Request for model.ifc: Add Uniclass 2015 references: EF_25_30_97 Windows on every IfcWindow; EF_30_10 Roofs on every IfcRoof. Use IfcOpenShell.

First a look at what the model holds.

```python
import ifcopenshell

model = ifcopenshell.open("model.ifc")
print(model.schema)
print("classifications:", [c.Name for c in model.by_type("IfcClassification")])
for ifc_class in ("IfcDoor", "IfcRoof", "IfcStair", "IfcWall", "IfcWindow"):
    print(ifc_class, len(model.by_type(ifc_class)))
```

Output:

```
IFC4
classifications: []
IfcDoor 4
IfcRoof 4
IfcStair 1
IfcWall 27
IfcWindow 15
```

```python
import ifcopenshell
import ifcopenshell.api.classification

model = ifcopenshell.open("model.ifc")

system = ifcopenshell.api.classification.add_classification(model, classification="Uniclass 2015")

codes = {
    "IfcWindow": ("EF_25_30_97", "Windows"),
    "IfcRoof": ("EF_30_10", "Roofs"),
}
for ifc_class, (code, name) in codes.items():
    products = model.by_type(ifc_class)
    ifcopenshell.api.classification.add_reference(
        model, products=products, classification=system, identification=code, name=name
    )
    print(code, len(products))

model.write("model_v2.ifc")
```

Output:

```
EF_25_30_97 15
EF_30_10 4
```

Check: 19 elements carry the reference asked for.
